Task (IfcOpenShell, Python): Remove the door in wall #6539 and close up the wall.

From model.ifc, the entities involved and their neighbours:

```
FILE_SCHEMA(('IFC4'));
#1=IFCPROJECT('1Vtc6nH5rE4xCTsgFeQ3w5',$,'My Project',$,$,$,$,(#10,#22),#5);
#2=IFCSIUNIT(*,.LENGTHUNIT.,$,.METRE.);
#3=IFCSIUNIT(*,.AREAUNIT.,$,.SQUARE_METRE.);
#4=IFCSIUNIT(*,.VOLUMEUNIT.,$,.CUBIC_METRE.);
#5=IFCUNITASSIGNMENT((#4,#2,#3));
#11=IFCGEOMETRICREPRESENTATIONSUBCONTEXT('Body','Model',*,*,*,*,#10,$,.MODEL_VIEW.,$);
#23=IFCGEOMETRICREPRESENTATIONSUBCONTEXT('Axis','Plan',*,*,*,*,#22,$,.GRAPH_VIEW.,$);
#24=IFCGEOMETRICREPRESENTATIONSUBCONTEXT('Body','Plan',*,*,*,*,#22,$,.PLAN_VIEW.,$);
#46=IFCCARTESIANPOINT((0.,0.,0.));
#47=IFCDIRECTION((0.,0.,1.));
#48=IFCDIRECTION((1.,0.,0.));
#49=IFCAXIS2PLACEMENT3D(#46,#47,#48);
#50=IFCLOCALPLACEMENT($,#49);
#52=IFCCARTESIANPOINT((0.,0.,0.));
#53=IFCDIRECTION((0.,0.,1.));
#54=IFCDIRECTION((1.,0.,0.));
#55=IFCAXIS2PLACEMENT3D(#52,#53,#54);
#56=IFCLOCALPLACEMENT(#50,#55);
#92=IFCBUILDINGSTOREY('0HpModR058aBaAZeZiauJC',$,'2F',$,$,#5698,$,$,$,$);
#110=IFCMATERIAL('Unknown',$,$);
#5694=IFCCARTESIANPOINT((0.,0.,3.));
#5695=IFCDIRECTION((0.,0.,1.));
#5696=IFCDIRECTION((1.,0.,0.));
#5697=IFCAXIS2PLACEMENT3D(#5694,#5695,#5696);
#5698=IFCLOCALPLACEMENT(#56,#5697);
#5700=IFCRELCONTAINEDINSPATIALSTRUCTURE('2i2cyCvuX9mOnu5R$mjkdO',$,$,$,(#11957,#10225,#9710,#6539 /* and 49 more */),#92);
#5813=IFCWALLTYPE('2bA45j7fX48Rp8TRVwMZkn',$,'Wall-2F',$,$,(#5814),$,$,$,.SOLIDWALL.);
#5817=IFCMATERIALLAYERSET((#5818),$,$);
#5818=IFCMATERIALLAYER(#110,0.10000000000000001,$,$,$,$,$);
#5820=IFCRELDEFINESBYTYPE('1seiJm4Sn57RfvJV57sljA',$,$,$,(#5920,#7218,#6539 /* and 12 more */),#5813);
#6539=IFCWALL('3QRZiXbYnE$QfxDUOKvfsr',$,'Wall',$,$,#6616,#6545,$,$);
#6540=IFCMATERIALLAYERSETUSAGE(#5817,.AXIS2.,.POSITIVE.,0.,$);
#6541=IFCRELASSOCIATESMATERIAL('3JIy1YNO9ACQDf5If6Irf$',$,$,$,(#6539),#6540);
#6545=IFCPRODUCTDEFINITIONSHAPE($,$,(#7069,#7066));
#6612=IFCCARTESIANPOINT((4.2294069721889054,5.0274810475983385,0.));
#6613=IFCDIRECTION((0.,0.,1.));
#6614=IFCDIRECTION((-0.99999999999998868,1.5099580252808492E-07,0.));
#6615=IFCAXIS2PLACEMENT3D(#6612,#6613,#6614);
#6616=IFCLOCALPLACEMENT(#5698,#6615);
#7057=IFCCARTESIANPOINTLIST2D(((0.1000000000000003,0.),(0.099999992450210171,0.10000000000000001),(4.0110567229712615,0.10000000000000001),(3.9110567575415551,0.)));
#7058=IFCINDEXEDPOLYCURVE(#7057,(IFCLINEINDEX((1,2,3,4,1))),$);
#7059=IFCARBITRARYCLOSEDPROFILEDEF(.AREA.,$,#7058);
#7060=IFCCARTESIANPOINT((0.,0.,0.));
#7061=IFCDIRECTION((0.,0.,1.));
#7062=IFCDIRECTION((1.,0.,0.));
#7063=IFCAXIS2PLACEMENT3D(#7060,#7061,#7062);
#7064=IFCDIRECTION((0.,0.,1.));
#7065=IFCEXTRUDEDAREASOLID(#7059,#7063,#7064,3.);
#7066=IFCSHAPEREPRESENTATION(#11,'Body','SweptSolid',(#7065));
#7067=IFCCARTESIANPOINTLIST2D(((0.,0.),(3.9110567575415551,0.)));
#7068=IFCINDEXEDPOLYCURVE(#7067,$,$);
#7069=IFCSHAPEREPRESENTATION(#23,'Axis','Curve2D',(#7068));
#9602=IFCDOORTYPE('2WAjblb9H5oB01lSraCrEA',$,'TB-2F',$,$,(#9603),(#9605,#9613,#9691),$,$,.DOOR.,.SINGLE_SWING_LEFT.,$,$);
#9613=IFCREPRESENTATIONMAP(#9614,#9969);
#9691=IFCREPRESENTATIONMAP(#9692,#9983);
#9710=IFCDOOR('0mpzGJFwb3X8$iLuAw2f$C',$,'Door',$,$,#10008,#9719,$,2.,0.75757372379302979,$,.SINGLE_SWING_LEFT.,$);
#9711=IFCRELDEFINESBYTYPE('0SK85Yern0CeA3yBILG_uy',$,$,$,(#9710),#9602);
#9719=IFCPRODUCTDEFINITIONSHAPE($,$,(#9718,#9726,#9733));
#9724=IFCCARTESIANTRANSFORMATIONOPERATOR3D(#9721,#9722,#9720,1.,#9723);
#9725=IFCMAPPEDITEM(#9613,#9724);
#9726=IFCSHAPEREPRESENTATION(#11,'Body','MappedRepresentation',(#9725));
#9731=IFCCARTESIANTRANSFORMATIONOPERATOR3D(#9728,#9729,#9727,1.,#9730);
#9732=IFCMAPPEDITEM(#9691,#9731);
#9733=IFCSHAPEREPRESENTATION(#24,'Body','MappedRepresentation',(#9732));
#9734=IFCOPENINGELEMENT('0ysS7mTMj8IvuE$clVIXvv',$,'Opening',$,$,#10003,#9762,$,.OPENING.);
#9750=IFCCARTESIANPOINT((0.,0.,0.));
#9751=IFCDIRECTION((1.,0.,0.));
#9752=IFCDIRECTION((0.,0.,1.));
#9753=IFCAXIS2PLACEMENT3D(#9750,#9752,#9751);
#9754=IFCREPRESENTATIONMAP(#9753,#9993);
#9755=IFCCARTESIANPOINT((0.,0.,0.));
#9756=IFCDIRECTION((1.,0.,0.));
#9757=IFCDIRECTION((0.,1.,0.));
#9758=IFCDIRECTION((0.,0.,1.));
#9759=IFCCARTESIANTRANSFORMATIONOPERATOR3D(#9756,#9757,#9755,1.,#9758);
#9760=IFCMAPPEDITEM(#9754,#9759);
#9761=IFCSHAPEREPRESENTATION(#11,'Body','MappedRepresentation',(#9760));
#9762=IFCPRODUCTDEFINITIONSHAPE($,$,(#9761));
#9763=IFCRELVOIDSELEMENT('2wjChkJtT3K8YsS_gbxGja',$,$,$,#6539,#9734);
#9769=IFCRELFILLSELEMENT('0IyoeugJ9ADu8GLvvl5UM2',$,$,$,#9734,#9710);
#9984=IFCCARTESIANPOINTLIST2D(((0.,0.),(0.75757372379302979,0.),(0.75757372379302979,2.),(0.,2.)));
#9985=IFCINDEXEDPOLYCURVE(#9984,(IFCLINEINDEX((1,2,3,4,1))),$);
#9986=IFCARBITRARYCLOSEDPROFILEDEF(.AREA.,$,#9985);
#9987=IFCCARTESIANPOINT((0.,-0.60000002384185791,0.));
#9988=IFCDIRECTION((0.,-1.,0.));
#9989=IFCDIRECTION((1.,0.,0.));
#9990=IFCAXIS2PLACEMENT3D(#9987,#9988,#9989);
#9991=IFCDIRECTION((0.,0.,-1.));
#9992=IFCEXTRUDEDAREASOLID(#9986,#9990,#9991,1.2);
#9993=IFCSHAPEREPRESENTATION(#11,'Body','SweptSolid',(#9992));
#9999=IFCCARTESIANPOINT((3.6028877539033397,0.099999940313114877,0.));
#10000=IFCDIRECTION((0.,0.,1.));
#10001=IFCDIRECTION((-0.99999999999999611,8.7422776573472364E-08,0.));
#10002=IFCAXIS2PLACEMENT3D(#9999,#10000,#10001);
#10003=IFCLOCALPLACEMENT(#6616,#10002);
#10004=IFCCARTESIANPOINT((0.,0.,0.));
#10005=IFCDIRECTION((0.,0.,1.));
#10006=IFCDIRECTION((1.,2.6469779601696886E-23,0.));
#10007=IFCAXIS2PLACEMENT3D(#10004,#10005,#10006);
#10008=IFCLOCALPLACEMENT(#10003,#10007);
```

```python
import ifcopenshell
import ifcopenshell.api.feature
import ifcopenshell.api.root
import ifcopenshell.geom
import ifcopenshell.util.shape

model = ifcopenshell.open("model.ifc")
settings = ifcopenshell.geom.settings()


def volume(element):
    """Net volume in cubic metres, openings subtracted."""
    shape = ifcopenshell.geom.create_shape(settings, element)
    return ifcopenshell.util.shape.get_volume(shape.geometry)


door = model.by_id(9710)
opening = door.FillsVoids[0].RelatingOpeningElement
wall = opening.VoidsElements[0].RelatingBuildingElement
before = volume(wall)

ifcopenshell.api.root.remove_product(model, product=door)
ifcopenshell.api.feature.remove_feature(model, feature=opening)

after = volume(wall)

print(f"wall volume {before:.3f} -> {after:.3f} m3")

model.write("model-out.ifc")
```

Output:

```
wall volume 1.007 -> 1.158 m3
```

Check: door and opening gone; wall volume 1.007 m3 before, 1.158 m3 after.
